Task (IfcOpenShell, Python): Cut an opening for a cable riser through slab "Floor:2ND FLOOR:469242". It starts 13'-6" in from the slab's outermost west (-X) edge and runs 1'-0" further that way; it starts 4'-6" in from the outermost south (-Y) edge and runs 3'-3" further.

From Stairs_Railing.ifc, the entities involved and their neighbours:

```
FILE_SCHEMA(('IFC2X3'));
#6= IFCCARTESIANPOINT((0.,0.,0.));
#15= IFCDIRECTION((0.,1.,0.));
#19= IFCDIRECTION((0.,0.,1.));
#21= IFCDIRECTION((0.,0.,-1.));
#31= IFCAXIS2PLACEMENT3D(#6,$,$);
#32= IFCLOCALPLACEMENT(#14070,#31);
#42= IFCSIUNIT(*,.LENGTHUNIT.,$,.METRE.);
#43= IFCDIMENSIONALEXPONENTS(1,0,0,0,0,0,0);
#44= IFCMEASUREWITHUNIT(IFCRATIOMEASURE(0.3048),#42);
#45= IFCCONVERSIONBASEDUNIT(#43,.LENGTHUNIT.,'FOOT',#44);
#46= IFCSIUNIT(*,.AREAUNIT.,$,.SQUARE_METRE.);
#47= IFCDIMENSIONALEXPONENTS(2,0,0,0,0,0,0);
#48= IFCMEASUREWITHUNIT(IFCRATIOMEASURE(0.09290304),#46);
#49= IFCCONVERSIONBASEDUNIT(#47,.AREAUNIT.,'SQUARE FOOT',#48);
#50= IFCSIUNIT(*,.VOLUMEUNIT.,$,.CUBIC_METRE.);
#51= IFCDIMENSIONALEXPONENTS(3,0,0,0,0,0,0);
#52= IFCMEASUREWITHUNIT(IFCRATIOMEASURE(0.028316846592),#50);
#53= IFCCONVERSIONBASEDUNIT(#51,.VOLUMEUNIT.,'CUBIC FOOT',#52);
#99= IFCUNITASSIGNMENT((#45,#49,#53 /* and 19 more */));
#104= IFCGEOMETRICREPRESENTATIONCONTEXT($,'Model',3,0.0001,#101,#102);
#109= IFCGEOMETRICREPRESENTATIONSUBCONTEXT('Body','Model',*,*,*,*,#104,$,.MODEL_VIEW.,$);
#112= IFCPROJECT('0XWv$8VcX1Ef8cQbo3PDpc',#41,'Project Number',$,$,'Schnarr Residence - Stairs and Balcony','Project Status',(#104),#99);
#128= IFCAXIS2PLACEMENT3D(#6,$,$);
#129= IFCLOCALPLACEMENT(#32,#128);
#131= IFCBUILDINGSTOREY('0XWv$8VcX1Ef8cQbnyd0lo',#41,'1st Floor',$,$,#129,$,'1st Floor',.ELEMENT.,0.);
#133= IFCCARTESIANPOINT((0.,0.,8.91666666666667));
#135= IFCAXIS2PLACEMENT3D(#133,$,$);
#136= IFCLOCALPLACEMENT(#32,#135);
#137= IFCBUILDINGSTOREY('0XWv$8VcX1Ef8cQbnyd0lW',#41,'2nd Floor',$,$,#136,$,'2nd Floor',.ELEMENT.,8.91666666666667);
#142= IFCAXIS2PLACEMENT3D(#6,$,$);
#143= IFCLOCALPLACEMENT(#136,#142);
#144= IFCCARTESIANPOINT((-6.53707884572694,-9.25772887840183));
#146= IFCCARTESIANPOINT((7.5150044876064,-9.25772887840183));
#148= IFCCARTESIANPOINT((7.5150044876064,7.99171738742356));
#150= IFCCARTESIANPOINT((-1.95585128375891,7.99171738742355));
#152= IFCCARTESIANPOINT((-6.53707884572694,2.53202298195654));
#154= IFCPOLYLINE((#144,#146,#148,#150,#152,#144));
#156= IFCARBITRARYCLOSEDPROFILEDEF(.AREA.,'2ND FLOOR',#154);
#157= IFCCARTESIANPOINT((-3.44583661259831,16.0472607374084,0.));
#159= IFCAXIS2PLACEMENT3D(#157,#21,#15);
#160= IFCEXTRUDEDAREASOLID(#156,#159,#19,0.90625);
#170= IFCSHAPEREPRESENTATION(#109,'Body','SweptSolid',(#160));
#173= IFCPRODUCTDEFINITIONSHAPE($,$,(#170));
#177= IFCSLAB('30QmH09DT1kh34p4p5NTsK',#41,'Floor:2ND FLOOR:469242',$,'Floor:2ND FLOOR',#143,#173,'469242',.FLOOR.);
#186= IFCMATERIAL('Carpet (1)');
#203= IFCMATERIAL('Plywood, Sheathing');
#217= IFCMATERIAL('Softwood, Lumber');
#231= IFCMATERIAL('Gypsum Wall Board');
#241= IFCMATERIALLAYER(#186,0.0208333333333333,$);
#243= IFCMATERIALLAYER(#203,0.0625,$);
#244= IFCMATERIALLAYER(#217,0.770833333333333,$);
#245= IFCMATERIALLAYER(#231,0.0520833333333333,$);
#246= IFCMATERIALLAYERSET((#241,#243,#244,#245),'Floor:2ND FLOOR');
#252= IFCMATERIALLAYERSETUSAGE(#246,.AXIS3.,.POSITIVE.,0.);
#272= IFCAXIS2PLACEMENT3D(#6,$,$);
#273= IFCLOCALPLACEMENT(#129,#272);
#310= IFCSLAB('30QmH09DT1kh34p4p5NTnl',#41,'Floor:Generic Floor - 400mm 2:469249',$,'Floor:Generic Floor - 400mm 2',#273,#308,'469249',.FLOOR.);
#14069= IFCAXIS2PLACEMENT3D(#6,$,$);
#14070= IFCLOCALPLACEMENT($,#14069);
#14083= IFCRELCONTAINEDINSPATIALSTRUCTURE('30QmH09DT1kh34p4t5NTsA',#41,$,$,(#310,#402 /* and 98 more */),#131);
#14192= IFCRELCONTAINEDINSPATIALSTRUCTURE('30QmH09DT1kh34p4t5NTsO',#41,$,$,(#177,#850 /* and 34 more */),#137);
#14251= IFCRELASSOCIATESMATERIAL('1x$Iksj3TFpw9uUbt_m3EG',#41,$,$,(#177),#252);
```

```python
import numpy as np
import ifcopenshell
import ifcopenshell.api.feature
import ifcopenshell.api.geometry
import ifcopenshell.api.root
import ifcopenshell.geom
import ifcopenshell.util.placement
import ifcopenshell.util.representation
import ifcopenshell.util.shape
import ifcopenshell.util.unit

model = ifcopenshell.open("Stairs_Railing.ifc")
unit_scale = ifcopenshell.util.unit.calculate_unit_scale(model)
settings = ifcopenshell.geom.settings()


def volume(element):
    """Net volume in cubic metres, openings subtracted."""
    shape = ifcopenshell.geom.create_shape(settings, element)
    return ifcopenshell.util.shape.get_volume(shape.geometry)


slab = model.by_id(177)
before = volume(slab)

# Extent in the slab's own axes, in metres. The edges named are its -X and -Y sides.
slab_shape = ifcopenshell.geom.create_shape(settings, slab)
vertices = ifcopenshell.util.shape.get_vertices(slab_shape.geometry)
x_min, y_min, bottom = vertices.min(axis=0)
top = vertices[:, 2].max()

opening = ifcopenshell.api.root.create_entity(model, ifc_class="IfcOpeningElement", name="Cable riser opening")
context = ifcopenshell.util.representation.get_context(model, "Model", "Body", "MODEL_VIEW")
width, depth = 0.3048, 0.9906
outline = [(0.0, 0.0), (width, 0.0), (width, depth), (0.0, depth), (0.0, 0.0)]
# Overshoot both faces by 50 mm so the cut is clean.
shape = ifcopenshell.api.geometry.add_slab_representation(
    model, context=context, depth=top - bottom + 0.1, polyline=outline
)
ifcopenshell.api.geometry.assign_representation(model, product=opening, representation=shape)

matrix = ifcopenshell.util.placement.get_local_placement(slab.ObjectPlacement)
matrix[:, 3] = matrix @ np.append(np.array([x_min + 4.1148, y_min + 1.3716, bottom - 0.05]) / unit_scale, 1.0)
ifcopenshell.api.geometry.edit_object_placement(model, product=opening, matrix=matrix, is_si=False)
ifcopenshell.api.feature.add_feature(model, feature=opening, element=slab)

after = volume(slab)

print(f"slab volume {before:.3f} -> {after:.3f} m3")

model.write("Stairs_Railing_edited.ifc")
```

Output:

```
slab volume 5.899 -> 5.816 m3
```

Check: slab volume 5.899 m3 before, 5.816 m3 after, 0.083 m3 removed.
